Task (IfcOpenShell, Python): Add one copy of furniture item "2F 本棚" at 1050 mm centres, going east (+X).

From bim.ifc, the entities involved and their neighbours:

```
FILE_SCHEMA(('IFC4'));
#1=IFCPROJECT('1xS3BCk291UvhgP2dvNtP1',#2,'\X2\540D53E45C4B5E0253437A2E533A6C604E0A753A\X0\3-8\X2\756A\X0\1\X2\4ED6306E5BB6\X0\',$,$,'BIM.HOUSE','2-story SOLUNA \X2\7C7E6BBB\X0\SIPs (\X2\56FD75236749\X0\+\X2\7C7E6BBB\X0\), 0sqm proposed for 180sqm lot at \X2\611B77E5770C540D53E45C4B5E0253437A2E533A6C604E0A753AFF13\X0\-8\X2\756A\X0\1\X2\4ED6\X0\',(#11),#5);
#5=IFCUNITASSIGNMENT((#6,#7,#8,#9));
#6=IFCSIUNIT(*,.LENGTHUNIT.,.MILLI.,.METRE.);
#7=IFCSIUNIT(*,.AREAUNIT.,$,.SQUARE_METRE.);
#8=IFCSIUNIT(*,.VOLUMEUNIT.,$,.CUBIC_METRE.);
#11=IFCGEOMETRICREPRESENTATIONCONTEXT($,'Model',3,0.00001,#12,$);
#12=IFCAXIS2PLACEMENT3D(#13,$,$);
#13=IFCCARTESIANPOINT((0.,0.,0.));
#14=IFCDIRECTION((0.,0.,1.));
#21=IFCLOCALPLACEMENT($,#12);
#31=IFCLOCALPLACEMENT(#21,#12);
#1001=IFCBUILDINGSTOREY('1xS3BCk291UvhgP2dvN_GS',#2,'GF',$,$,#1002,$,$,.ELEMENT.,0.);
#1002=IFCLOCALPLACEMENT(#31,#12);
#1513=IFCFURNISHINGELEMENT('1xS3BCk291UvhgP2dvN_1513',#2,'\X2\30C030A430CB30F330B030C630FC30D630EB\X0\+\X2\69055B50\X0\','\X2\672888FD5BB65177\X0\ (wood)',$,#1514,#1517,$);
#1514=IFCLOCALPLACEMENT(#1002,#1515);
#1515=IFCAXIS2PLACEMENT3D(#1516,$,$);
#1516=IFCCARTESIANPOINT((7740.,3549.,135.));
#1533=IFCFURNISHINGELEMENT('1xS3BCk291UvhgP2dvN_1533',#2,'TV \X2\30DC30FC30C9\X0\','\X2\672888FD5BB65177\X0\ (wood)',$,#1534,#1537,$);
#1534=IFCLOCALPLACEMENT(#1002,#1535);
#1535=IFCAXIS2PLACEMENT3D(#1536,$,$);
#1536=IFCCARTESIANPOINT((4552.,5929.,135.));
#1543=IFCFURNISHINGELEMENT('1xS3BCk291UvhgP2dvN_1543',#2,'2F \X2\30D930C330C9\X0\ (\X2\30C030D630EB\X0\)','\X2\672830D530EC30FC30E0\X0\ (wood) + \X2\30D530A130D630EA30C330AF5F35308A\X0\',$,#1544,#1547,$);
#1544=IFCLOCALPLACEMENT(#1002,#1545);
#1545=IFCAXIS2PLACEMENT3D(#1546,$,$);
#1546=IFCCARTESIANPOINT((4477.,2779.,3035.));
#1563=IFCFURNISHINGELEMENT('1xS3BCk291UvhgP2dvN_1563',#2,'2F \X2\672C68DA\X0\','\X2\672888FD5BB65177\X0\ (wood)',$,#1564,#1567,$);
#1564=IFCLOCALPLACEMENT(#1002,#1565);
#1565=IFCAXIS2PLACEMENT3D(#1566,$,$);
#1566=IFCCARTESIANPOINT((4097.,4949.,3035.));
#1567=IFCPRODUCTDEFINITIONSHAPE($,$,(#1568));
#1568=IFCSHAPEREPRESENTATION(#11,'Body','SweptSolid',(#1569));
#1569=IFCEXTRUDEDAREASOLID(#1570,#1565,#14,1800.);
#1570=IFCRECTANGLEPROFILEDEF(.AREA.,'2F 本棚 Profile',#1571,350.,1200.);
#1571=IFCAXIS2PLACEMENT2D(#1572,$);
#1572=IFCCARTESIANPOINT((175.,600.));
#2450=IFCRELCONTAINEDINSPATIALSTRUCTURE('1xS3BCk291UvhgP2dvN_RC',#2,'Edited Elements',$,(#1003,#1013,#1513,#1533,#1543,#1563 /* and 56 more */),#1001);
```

```python
import numpy as np
import ifcopenshell
import ifcopenshell.api.geometry
import ifcopenshell.api.root
import ifcopenshell.util.element
import ifcopenshell.util.placement

model = ifcopenshell.open("bim.ifc")


def reuse_history(source, copy):
    """copy_class also copies each property set's owner history, people and application; keep the originals."""
    for rel in copy.IsDefinedBy:
        if rel.is_a("IfcRelDefinesByProperties") and (history := rel.RelatingPropertyDefinition.OwnerHistory):
            rel.RelatingPropertyDefinition.OwnerHistory = source.OwnerHistory
            ifcopenshell.util.element.remove_deep2(model, history)


source = model.by_guid("1xS3BCk291UvhgP2dvN_1563")
base = ifcopenshell.util.placement.get_local_placement(source.ObjectPlacement)
step = np.array([1.0, 0.0, 0.0]) * 1050.0

for i in range(1, 2):
    copy = ifcopenshell.api.root.copy_class(model, product=source)
    copy.Representation = ifcopenshell.util.element.copy_deep(
        model, source.Representation, exclude=["IfcGeometricRepresentationContext", "IfcRepresentationMap"]
    )
    reuse_history(source, copy)
    matrix = base.copy()
    matrix[:3, 3] += i * step
    print("added at", matrix[:3, 3].round(3) + 0.0)
    ifcopenshell.api.geometry.edit_object_placement(model, product=copy, matrix=matrix, is_si=False)

model.write("bim_edited.ifc")
```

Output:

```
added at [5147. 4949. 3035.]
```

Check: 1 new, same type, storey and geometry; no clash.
